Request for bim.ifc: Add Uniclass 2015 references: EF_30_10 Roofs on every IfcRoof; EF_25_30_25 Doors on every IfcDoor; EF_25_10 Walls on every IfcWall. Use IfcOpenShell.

First a look at what the model holds.

```python
import ifcopenshell

model = ifcopenshell.open("bim.ifc")
print(model.schema)
print("classifications:", [c.Name for c in model.by_type("IfcClassification")])
for ifc_class in ("IfcDoor", "IfcRoof", "IfcStair", "IfcWall", "IfcWindow"):
    print(ifc_class, len(model.by_type(ifc_class)))
```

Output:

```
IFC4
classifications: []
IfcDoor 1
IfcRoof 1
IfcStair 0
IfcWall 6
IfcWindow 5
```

```python
import ifcopenshell
import ifcopenshell.api.classification

model = ifcopenshell.open("bim.ifc")

system = ifcopenshell.api.classification.add_classification(model, classification="Uniclass 2015")

codes = {
    "IfcRoof": ("EF_30_10", "Roofs"),
    "IfcDoor": ("EF_25_30_25", "Doors"),
    "IfcWall": ("EF_25_10", "Walls"),
}
for ifc_class, (code, name) in codes.items():
    products = model.by_type(ifc_class)
    ifcopenshell.api.classification.add_reference(
        model, products=products, classification=system, identification=code, name=name
    )
    print(code, len(products))

model.write("bim_updated.ifc")
```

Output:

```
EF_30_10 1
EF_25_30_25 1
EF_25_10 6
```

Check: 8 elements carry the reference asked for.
